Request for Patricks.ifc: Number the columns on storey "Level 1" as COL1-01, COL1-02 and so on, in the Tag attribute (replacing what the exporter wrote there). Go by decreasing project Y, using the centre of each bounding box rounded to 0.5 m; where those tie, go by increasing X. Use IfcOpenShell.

First a look at what the model holds.

```python
import ifcopenshell
import ifcopenshell.util.element
import ifcopenshell.util.placement

model = ifcopenshell.open("Patricks.ifc")
print(model.schema)
storey = next(s for s in model.by_type("IfcBuildingStorey") if s.Name == "Level 1")
columns = [e for e in ifcopenshell.util.element.get_decomposition(storey) if e.is_a("IfcColumn")]
for e in sorted(columns, key=lambda e: e.id()):
    origin = ifcopenshell.util.placement.get_local_placement(e.ObjectPlacement)[:3, 3]
    print(e.id(), e.Tag, e.Name, origin.round(2) + 0.0, sep=" | ")
```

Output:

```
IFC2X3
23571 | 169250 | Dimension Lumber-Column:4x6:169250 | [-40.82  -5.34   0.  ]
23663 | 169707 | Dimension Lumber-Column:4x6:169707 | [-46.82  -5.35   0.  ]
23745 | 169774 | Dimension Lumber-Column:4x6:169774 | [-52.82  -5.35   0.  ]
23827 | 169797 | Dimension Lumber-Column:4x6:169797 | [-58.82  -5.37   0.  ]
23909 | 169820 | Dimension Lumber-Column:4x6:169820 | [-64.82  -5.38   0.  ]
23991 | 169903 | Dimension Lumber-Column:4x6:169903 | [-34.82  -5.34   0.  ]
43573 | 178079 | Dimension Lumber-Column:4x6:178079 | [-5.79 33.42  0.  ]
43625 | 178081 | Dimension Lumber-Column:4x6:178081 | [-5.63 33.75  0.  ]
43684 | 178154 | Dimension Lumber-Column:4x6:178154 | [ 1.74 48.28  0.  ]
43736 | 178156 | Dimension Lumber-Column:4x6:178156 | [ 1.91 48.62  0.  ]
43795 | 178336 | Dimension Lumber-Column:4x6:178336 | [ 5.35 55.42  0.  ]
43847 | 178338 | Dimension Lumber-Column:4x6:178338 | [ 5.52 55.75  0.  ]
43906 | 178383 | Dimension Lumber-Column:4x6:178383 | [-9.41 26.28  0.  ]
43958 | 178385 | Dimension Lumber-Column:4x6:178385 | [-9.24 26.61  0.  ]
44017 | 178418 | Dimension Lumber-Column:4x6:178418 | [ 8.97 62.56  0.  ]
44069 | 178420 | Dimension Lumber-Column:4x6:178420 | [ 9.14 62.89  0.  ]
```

```python
import ifcopenshell
import ifcopenshell.geom
import ifcopenshell.util.element
import ifcopenshell.util.shape

model = ifcopenshell.open("Patricks.ifc")
settings = ifcopenshell.geom.settings()
settings.set("use-world-coords", True)


def centre(element):
    shape = ifcopenshell.geom.create_shape(settings, element)
    return ifcopenshell.util.shape.get_bbox_centroid(shape.geometry)


storey = next(s for s in model.by_type("IfcBuildingStorey") if s.Name == "Level 1")
columns = [e for e in ifcopenshell.util.element.get_decomposition(storey) if e.is_a("IfcColumn")]

# Insertion points can sit at a corner or the storey origin, so sort by the geometry (in metres).
centres = {e: centre(e) for e in columns}
columns.sort(key=lambda e: (-round(centres[e][1] / 0.5), centres[e][0]))

for i, e in enumerate(columns, start=1):
    number = f"COL1-{i:02d}"
    e.Tag = number
    print(e.id(), number)

model.write("Patricks_rev.ifc")
```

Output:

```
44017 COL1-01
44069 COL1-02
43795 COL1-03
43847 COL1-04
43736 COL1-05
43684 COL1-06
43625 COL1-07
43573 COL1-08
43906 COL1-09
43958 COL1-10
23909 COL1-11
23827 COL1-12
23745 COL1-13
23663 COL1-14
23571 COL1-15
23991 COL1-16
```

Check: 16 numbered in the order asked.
